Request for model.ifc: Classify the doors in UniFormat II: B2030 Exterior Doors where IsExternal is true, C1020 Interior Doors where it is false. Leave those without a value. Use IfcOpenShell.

First a look at what the model holds.

```python
import ifcopenshell
import ifcopenshell.util.element

model = ifcopenshell.open("model.ifc")
print(model.schema)
print("classifications:", [c.Name for c in model.by_type("IfcClassification")])
values = [ifcopenshell.util.element.get_pset(e, "Pset_DoorCommon", "IsExternal") for e in model.by_type("IfcDoor")]
for value in (True, False, None):
    print("IsExternal", value, values.count(value))
```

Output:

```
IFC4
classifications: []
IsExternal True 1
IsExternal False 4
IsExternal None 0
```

```python
import ifcopenshell
import ifcopenshell.api.classification
import ifcopenshell.util.element

model = ifcopenshell.open("model.ifc")

system = ifcopenshell.api.classification.add_classification(model, classification="UniFormat II")

doors = model.by_type("IfcDoor")
external = {e: ifcopenshell.util.element.get_pset(e, "Pset_DoorCommon", "IsExternal") for e in doors}
for flag, code, name in ((True, "B2030", "Exterior Doors"), (False, "C1020", "Interior Doors")):
    products = [e for e in doors if external[e] is flag]
    ifcopenshell.api.classification.add_reference(
        model, products=products, classification=system, identification=code, name=name
    )
    print(code, len(products))

model.write("model_v2.ifc")
```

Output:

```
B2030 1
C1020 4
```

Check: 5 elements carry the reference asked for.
